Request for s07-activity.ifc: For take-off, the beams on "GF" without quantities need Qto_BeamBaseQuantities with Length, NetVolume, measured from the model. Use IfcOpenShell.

First a look at what the model holds.

```python
import ifcopenshell
import ifcopenshell.util.element
import ifcopenshell.util.unit

model = ifcopenshell.open("s07-activity.ifc")
print(model.schema)
for unit_type in ("LENGTHUNIT", "AREAUNIT", "VOLUMEUNIT"):
    print(unit_type, ifcopenshell.util.unit.calculate_unit_scale(model, unit_type))
storey = next(s for s in model.by_type("IfcBuildingStorey") if s.Name == "GF")
beams = [e for e in ifcopenshell.util.element.get_decomposition(storey) if e.is_a("IfcBeam")]
for e in sorted(beams, key=lambda e: e.id()):
    print(e.id(), e.is_a(), e.Name, list(ifcopenshell.util.element.get_psets(e, qtos_only=True)), sep=" | ")
```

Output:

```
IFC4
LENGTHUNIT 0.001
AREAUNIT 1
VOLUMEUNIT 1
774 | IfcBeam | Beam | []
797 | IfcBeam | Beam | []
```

```python
import ifcopenshell
import ifcopenshell.api.pset
import ifcopenshell.geom
import ifcopenshell.util.element
import ifcopenshell.util.shape
import ifcopenshell.util.unit

model = ifcopenshell.open("s07-activity.ifc")
unit_scale = ifcopenshell.util.unit.calculate_unit_scale(model)
volume_scale = ifcopenshell.util.unit.calculate_unit_scale(model, "VOLUMEUNIT")
settings = ifcopenshell.geom.settings()

storey = next(s for s in model.by_type("IfcBuildingStorey") if s.Name == "GF")
beams = [e for e in ifcopenshell.util.element.get_decomposition(storey) if e.is_a("IfcBeam")]

for e in sorted(beams, key=lambda e: e.id()):
    if ifcopenshell.util.element.get_psets(e, qtos_only=True, should_inherit=False):
        continue
    # Geometry comes back in metres, in the element's own axes.
    shape = ifcopenshell.geom.create_shape(settings, e)
    values = {
        "Length": ifcopenshell.util.shape.get_max_xyz(shape.geometry) / unit_scale,
        "NetVolume": ifcopenshell.util.shape.get_volume(shape.geometry) / volume_scale,
    }
    qto = ifcopenshell.api.pset.add_qto(model, product=e, name="Qto_BeamBaseQuantities")
    ifcopenshell.api.pset.edit_qto(model, qto=qto, properties=values)
    print(e.id(), {k: round(v, 3) for k, v in values.items()})

model.write("s07-activity_v2.ifc")
```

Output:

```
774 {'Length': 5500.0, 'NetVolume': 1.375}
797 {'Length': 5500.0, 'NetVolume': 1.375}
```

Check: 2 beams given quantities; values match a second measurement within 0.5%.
